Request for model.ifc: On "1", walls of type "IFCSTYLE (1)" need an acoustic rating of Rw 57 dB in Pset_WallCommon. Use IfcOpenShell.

First a look at what the model holds.

```python
import ifcopenshell
import ifcopenshell.util.element

model = ifcopenshell.open("model.ifc")
print(model.schema)
storey = next(s for s in model.by_type("IfcBuildingStorey") if s.Name == "1")
walls = [e for e in ifcopenshell.util.element.get_decomposition(storey) if e.is_a("IfcWall")]
seen = {}
for e in walls:
    element_type = ifcopenshell.util.element.get_type(e)
    key = (element_type.Name if element_type != e and element_type else None, ifcopenshell.util.element.get_pset(e, "Pset_WallCommon", "AcousticRating"))
    seen[key] = seen.get(key, 0) + 1
for (name, value), count in sorted(seen.items(), key=str):
    print(count, "x", name, "|", value)
```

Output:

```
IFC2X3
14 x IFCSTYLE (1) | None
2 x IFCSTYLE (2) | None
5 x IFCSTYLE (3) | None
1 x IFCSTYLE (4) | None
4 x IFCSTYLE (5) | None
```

```python
import ifcopenshell
import ifcopenshell.api.pset
import ifcopenshell.util.element

model = ifcopenshell.open("model.ifc")

storey = next(s for s in model.by_type("IfcBuildingStorey") if s.Name == "1")
walls = [e for e in ifcopenshell.util.element.get_decomposition(storey) if e.is_a("IfcWall")]

count = 0
for e in walls:
    element_type = ifcopenshell.util.element.get_type(e)
    if element_type in (None, e) or element_type.Name != "IFCSTYLE (1)":
        continue
    # add_pset returns the element's existing set when there is one.
    pset = ifcopenshell.api.pset.add_pset(model, product=e, name="Pset_WallCommon")
    ifcopenshell.api.pset.edit_pset(model, pset=pset, properties={"AcousticRating": "Rw 57 dB"})
    count += 1

print(count, "walls updated")

model.write("model_v2.ifc")
```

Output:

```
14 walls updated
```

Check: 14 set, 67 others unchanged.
